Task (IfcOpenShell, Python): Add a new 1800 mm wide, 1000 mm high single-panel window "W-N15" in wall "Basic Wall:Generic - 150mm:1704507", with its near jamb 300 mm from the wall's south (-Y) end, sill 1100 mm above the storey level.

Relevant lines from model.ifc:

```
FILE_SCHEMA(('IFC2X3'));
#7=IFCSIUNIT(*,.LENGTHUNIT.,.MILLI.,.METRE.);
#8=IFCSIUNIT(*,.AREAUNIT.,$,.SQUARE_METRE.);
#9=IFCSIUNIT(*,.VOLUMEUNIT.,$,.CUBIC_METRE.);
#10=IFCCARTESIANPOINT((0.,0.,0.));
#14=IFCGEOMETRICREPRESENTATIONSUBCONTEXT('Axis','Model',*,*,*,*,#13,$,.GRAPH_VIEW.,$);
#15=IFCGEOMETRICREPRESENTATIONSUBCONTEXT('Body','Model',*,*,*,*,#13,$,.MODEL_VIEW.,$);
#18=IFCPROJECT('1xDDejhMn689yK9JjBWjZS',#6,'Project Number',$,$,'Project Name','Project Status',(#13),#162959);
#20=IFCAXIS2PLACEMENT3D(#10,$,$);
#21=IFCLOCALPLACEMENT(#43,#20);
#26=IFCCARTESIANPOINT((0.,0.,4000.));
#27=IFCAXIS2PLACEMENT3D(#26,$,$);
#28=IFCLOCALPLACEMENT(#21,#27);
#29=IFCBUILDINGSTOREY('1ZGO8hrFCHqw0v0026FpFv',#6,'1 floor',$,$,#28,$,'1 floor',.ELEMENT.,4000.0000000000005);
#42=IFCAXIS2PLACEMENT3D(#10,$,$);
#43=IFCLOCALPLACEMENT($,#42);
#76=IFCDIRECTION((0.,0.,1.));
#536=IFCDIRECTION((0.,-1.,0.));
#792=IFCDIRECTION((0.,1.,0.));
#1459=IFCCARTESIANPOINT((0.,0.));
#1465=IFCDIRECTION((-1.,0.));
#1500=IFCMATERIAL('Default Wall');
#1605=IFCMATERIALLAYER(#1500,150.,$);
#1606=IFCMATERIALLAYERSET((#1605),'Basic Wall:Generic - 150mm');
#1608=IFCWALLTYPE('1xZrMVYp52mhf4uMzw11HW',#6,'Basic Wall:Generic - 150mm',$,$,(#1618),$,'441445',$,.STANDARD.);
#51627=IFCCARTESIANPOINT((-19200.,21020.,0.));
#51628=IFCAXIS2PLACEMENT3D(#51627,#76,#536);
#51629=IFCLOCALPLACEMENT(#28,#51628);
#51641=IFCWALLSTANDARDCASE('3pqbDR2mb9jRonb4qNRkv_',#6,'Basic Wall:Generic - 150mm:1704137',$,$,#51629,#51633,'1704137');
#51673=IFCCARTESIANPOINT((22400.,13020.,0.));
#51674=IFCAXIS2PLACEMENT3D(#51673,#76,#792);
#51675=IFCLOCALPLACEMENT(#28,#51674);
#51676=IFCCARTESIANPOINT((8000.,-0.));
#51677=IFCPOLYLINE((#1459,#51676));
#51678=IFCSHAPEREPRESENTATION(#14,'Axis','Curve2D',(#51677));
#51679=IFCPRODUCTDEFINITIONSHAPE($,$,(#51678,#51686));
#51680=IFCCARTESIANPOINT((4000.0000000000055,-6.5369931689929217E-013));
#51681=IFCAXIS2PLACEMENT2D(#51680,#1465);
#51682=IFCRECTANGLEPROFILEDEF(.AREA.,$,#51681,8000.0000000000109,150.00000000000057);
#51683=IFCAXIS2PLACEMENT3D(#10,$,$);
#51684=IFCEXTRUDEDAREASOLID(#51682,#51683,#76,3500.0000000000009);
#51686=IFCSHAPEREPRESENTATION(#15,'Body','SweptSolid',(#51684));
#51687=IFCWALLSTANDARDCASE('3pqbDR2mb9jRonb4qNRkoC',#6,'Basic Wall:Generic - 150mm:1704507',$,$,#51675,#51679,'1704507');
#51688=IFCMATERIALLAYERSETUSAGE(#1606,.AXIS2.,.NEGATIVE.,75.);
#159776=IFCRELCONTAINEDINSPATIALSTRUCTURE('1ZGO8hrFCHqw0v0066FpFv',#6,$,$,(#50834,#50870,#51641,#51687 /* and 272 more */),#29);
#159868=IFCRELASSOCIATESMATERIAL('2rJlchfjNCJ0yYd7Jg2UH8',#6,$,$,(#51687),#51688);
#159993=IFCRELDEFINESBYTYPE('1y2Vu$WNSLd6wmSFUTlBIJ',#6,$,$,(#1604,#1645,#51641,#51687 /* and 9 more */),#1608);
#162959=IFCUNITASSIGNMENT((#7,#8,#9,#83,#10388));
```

```python
import numpy as np
import ifcopenshell
import ifcopenshell.api.feature
import ifcopenshell.api.geometry
import ifcopenshell.api.root
import ifcopenshell.api.spatial
import ifcopenshell.api.type
import ifcopenshell.geom
import ifcopenshell.util.element
import ifcopenshell.util.placement
import ifcopenshell.util.representation
import ifcopenshell.util.shape
import ifcopenshell.util.unit

model = ifcopenshell.open("model.ifc")
unit_scale = ifcopenshell.util.unit.calculate_unit_scale(model)
settings = ifcopenshell.geom.settings()


def volume(element):
    """Net volume in cubic metres, openings subtracted."""
    shape = ifcopenshell.geom.create_shape(settings, element)
    return ifcopenshell.util.shape.get_volume(shape.geometry)


wall = model.by_guid("3pqbDR2mb9jRonb4qNRkoC")
storey = ifcopenshell.util.element.get_container(wall, ifc_class="IfcBuildingStorey")
context = ifcopenshell.util.representation.get_context(model, "Model", "Body", "MODEL_VIEW")
before = volume(wall)

width, height, from_end, sill = 1.8, 1, 0.3, 1.1  # metres

# The wall runs along its own X axis, and the end named is its -X end.
wall_shape = ifcopenshell.geom.create_shape(settings, wall)
x, y, z = ifcopenshell.util.shape.get_vertices(wall_shape.geometry).T
start = x.min() + from_end
face, thickness = float(y.min()), float(y.max() - y.min())
wall_matrix = ifcopenshell.util.placement.get_local_placement(wall.ObjectPlacement)
level = ifcopenshell.util.placement.get_local_placement(storey.ObjectPlacement)[2, 3]


def in_wall(x, y):
    """Placement at x, y metres in the wall's axes, at sill height."""
    matrix = wall_matrix.copy()
    matrix[:, 3] = wall_matrix @ np.array([x / unit_scale, y / unit_scale, 0.0, 1.0])
    matrix[2, 3] = level + sill / unit_scale
    return matrix


# Opening: a box that overshoots both wall faces by 50 mm.
opening = ifcopenshell.api.root.create_entity(model, ifc_class="IfcOpeningElement")
box = ifcopenshell.api.geometry.add_wall_representation(
    model, context=context, length=width, height=height, thickness=thickness + 0.1
)
ifcopenshell.api.geometry.assign_representation(model, product=opening, representation=box)
ifcopenshell.api.geometry.edit_object_placement(model, product=opening, matrix=in_wall(start, face - 0.05), is_si=False)
ifcopenshell.api.feature.add_feature(model, feature=opening, element=wall)

window = ifcopenshell.api.root.create_entity(model, ifc_class="IfcWindow", name="W-N15")
window.OverallWidth, window.OverallHeight = width / unit_scale, height / unit_scale
body = ifcopenshell.api.geometry.add_window_representation(
    model,
    context=context,
    overall_width=window.OverallWidth,
    overall_height=window.OverallHeight,
    partition_type="SINGLE_PANEL",
)
ifcopenshell.api.geometry.assign_representation(model, product=window, representation=body)
ifcopenshell.api.spatial.assign_container(model, products=[window], relating_structure=storey)
fills = ifcopenshell.api.feature.add_filling(model, opening=opening, element=window)
fills.OwnerHistory = window.OwnerHistory  # required in IFC2X3

# IFC2X3 keeps the operation on the window style.
style = ifcopenshell.api.root.create_entity(model, ifc_class="IfcWindowStyle", name="W-N15")
style.OperationType, style.ConstructionType = "SINGLE_PANEL", "NOTDEFINED"
style.ParameterTakesPrecedence = style.Sizeable = False
ifcopenshell.api.type.assign_type(model, related_objects=[window], relating_type=style)

# Centre the window in the wall's thickness.
ifcopenshell.api.geometry.edit_object_placement(model, product=window, matrix=in_wall(start, face), is_si=False)
window_shape = ifcopenshell.geom.create_shape(settings, window)
depth = ifcopenshell.util.shape.get_vertices(window_shape.geometry)[:, 1]
offset = face + thickness / 2 - (depth.min() + depth.max()) / 2
ifcopenshell.api.geometry.edit_object_placement(model, product=window, matrix=in_wall(start, offset), is_si=False)

after = volume(wall)

print(f"wall volume {before:.3f} -> {after:.3f} m3")

model.write("model_rev.ifc")
```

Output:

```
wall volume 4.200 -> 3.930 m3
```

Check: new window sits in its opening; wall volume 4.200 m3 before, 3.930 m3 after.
